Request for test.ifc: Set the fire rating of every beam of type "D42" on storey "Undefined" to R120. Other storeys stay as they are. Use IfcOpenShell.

First a look at what the model holds.

```python
import ifcopenshell
import ifcopenshell.util.element

model = ifcopenshell.open("test.ifc")
print(model.schema)
storey = next(s for s in model.by_type("IfcBuildingStorey") if s.Name == "Undefined")
beams = [e for e in ifcopenshell.util.element.get_decomposition(storey) if e.is_a("IfcBeam")]
seen = {}
for e in beams:
    element_type = ifcopenshell.util.element.get_type(e)
    key = (element_type.Name if element_type != e and element_type else None, ifcopenshell.util.element.get_pset(e, "Pset_BeamCommon", "FireRating"))
    seen[key] = seen.get(key, 0) + 1
for (name, value), count in sorted(seen.items(), key=str):
    print(count, "x", name, "|", value)
```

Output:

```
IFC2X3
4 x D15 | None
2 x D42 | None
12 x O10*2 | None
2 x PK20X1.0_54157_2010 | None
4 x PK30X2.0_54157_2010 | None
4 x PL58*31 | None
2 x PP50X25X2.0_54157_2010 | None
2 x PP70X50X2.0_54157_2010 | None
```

```python
import ifcopenshell
import ifcopenshell.api.pset
import ifcopenshell.util.element

model = ifcopenshell.open("test.ifc")

storey = next(s for s in model.by_type("IfcBuildingStorey") if s.Name == "Undefined")
beams = [e for e in ifcopenshell.util.element.get_decomposition(storey) if e.is_a("IfcBeam")]

count = 0
for e in beams:
    element_type = ifcopenshell.util.element.get_type(e)
    if element_type in (None, e) or element_type.Name != "D42":
        continue
    found = ifcopenshell.util.element.get_pset(e, "Pset_BeamCommon", should_inherit=False)
    if found:
        pset = model.by_id(found["id"])
        if len(ifcopenshell.util.element.get_elements_by_pset(pset)) > 1:
            pset = ifcopenshell.api.pset.unshare_pset(model, products=[e], pset=pset)[0]
    else:
        pset = ifcopenshell.api.pset.add_pset(model, product=e, name="Pset_BeamCommon")
    ifcopenshell.api.pset.edit_pset(model, pset=pset, properties={"FireRating": "R120"})
    count += 1

print(count, "beams updated")

model.write("test_v2.ifc")
```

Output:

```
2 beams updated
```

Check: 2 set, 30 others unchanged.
